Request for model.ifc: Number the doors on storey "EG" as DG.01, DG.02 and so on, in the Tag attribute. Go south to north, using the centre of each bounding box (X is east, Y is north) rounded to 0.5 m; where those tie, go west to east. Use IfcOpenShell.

First a look at what the model holds.

```python
import ifcopenshell
import ifcopenshell.util.element
import ifcopenshell.util.placement

model = ifcopenshell.open("model.ifc")
print(model.schema)
storey = next(s for s in model.by_type("IfcBuildingStorey") if s.Name == "EG")
doors = [e for e in ifcopenshell.util.element.get_decomposition(storey) if e.is_a("IfcDoor")]
for e in sorted(doors, key=lambda e: e.id()):
    origin = ifcopenshell.util.placement.get_local_placement(e.ObjectPlacement)[:3, 3]
    print(e.id(), e.Tag, e.Name, origin.round(2) + 0.0, sep=" | ")
```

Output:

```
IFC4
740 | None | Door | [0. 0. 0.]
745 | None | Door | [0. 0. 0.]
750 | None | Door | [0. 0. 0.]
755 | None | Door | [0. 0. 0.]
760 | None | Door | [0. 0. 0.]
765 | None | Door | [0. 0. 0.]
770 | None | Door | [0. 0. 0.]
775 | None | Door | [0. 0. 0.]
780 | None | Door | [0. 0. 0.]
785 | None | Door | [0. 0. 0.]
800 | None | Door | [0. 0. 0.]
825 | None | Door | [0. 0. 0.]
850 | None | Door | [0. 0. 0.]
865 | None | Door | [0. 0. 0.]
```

```python
import ifcopenshell
import ifcopenshell.geom
import ifcopenshell.util.element
import ifcopenshell.util.shape

model = ifcopenshell.open("model.ifc")
settings = ifcopenshell.geom.settings()
settings.set("use-world-coords", True)


def centre(element):
    shape = ifcopenshell.geom.create_shape(settings, element)
    return ifcopenshell.util.shape.get_bbox_centroid(shape.geometry)


storey = next(s for s in model.by_type("IfcBuildingStorey") if s.Name == "EG")
doors = [e for e in ifcopenshell.util.element.get_decomposition(storey) if e.is_a("IfcDoor")]

# Insertion points can sit at a corner or the storey origin, so sort by the geometry (in metres).
centres = {e: centre(e) for e in doors}
doors.sort(key=lambda e: (round(centres[e][1] / 0.5), centres[e][0]))

for i, e in enumerate(doors, start=1):
    number = f"DG.{i:02d}"
    e.Tag = number
    print(e.id(), number)

model.write("model-out.ifc")
```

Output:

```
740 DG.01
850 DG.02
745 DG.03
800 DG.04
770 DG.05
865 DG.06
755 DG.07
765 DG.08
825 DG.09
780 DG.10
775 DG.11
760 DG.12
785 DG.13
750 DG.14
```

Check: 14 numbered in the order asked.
